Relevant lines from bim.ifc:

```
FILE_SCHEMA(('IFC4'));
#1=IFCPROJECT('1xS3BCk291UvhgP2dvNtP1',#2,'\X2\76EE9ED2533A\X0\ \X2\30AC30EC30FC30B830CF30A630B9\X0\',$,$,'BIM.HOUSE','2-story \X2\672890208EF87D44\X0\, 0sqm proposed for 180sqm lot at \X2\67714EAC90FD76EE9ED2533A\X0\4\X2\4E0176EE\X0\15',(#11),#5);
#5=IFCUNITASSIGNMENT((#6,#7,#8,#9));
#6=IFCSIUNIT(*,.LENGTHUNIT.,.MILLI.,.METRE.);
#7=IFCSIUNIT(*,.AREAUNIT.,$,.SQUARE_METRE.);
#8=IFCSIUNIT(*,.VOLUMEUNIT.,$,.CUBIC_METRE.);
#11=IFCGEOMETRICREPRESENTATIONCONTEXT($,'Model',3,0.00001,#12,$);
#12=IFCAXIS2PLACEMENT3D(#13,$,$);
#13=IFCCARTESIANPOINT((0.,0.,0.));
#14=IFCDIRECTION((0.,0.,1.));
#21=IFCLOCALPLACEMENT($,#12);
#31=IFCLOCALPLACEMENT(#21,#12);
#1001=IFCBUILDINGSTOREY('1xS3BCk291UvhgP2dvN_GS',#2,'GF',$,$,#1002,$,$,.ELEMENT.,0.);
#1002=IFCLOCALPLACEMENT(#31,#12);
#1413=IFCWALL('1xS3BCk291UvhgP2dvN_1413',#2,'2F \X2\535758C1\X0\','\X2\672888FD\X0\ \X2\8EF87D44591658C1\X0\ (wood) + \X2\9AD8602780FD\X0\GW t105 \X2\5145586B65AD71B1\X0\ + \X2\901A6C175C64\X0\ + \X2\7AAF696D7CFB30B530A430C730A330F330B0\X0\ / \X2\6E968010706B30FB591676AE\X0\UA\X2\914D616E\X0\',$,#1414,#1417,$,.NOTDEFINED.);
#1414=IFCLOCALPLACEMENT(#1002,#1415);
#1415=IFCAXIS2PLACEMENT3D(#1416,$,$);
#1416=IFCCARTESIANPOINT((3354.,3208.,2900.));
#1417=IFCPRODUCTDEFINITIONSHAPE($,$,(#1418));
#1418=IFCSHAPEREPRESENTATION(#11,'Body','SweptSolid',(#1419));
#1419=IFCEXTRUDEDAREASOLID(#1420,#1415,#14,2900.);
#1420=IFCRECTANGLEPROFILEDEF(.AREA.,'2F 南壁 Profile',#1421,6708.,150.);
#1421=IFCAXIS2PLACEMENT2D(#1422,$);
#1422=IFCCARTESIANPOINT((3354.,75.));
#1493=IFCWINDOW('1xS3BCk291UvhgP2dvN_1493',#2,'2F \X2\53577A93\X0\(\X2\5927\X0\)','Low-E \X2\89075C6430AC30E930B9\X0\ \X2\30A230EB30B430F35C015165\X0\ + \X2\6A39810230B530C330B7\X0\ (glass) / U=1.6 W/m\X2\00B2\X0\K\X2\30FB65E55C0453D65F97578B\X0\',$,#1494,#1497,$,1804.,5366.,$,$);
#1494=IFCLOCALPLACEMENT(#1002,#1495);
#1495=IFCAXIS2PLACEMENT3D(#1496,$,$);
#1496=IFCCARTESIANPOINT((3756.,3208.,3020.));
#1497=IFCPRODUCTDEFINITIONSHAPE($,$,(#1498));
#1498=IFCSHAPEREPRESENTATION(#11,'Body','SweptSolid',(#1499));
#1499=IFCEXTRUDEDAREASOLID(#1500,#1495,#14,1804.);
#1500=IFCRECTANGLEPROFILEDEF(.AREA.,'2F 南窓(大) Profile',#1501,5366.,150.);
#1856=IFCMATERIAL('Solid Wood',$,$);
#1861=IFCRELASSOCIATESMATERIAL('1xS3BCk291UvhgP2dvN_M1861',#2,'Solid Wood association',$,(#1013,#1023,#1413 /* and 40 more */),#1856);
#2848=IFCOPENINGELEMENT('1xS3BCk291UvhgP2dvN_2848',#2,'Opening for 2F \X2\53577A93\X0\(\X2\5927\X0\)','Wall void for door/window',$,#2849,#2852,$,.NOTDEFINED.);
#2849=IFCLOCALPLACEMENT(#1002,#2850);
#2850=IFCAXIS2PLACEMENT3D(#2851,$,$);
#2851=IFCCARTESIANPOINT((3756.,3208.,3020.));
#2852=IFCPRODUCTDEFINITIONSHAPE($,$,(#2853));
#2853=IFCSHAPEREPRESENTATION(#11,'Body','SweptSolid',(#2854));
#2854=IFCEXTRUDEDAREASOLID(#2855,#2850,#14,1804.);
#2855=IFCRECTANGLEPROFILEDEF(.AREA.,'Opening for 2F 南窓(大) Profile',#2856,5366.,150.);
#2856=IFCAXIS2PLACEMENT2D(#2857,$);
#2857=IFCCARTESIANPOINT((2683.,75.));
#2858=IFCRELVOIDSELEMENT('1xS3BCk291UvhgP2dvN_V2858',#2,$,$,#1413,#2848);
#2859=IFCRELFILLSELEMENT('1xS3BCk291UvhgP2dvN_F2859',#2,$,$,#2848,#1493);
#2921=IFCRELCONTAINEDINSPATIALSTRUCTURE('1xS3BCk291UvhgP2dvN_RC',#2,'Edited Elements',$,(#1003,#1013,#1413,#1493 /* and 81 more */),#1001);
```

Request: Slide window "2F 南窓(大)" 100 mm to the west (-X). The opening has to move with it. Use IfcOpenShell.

```python
import ifcopenshell
import ifcopenshell.api.geometry
import ifcopenshell.util.placement
import ifcopenshell.util.unit

model = ifcopenshell.open("bim.ifc")
unit_scale = ifcopenshell.util.unit.calculate_unit_scale(model)

window = model.by_guid("1xS3BCk291UvhgP2dvN_1493")
opening = window.FillsVoids[0].RelatingOpeningElement
wall = opening.VoidsElements[0].RelatingBuildingElement

wall_matrix = ifcopenshell.util.placement.get_local_placement(wall.ObjectPlacement)
shift = wall_matrix[:3, 0] * -0.1 / unit_scale
before = ifcopenshell.util.placement.get_local_placement(window.ObjectPlacement)[:3, 3].copy()

# The window is not placed relative to its opening, so move both.
for product in (opening, window):
    matrix = ifcopenshell.util.placement.get_local_placement(product.ObjectPlacement)
    matrix[:3, 3] += shift
    ifcopenshell.api.geometry.edit_object_placement(model, product=product, matrix=matrix, is_si=False)

after = ifcopenshell.util.placement.get_local_placement(window.ObjectPlacement)[:3, 3]
print("window moved by", (after - before).round(3) + 0.0)

model.write("bim_rev.ifc")
```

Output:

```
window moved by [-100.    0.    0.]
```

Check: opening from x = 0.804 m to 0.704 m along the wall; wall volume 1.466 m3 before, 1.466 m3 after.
